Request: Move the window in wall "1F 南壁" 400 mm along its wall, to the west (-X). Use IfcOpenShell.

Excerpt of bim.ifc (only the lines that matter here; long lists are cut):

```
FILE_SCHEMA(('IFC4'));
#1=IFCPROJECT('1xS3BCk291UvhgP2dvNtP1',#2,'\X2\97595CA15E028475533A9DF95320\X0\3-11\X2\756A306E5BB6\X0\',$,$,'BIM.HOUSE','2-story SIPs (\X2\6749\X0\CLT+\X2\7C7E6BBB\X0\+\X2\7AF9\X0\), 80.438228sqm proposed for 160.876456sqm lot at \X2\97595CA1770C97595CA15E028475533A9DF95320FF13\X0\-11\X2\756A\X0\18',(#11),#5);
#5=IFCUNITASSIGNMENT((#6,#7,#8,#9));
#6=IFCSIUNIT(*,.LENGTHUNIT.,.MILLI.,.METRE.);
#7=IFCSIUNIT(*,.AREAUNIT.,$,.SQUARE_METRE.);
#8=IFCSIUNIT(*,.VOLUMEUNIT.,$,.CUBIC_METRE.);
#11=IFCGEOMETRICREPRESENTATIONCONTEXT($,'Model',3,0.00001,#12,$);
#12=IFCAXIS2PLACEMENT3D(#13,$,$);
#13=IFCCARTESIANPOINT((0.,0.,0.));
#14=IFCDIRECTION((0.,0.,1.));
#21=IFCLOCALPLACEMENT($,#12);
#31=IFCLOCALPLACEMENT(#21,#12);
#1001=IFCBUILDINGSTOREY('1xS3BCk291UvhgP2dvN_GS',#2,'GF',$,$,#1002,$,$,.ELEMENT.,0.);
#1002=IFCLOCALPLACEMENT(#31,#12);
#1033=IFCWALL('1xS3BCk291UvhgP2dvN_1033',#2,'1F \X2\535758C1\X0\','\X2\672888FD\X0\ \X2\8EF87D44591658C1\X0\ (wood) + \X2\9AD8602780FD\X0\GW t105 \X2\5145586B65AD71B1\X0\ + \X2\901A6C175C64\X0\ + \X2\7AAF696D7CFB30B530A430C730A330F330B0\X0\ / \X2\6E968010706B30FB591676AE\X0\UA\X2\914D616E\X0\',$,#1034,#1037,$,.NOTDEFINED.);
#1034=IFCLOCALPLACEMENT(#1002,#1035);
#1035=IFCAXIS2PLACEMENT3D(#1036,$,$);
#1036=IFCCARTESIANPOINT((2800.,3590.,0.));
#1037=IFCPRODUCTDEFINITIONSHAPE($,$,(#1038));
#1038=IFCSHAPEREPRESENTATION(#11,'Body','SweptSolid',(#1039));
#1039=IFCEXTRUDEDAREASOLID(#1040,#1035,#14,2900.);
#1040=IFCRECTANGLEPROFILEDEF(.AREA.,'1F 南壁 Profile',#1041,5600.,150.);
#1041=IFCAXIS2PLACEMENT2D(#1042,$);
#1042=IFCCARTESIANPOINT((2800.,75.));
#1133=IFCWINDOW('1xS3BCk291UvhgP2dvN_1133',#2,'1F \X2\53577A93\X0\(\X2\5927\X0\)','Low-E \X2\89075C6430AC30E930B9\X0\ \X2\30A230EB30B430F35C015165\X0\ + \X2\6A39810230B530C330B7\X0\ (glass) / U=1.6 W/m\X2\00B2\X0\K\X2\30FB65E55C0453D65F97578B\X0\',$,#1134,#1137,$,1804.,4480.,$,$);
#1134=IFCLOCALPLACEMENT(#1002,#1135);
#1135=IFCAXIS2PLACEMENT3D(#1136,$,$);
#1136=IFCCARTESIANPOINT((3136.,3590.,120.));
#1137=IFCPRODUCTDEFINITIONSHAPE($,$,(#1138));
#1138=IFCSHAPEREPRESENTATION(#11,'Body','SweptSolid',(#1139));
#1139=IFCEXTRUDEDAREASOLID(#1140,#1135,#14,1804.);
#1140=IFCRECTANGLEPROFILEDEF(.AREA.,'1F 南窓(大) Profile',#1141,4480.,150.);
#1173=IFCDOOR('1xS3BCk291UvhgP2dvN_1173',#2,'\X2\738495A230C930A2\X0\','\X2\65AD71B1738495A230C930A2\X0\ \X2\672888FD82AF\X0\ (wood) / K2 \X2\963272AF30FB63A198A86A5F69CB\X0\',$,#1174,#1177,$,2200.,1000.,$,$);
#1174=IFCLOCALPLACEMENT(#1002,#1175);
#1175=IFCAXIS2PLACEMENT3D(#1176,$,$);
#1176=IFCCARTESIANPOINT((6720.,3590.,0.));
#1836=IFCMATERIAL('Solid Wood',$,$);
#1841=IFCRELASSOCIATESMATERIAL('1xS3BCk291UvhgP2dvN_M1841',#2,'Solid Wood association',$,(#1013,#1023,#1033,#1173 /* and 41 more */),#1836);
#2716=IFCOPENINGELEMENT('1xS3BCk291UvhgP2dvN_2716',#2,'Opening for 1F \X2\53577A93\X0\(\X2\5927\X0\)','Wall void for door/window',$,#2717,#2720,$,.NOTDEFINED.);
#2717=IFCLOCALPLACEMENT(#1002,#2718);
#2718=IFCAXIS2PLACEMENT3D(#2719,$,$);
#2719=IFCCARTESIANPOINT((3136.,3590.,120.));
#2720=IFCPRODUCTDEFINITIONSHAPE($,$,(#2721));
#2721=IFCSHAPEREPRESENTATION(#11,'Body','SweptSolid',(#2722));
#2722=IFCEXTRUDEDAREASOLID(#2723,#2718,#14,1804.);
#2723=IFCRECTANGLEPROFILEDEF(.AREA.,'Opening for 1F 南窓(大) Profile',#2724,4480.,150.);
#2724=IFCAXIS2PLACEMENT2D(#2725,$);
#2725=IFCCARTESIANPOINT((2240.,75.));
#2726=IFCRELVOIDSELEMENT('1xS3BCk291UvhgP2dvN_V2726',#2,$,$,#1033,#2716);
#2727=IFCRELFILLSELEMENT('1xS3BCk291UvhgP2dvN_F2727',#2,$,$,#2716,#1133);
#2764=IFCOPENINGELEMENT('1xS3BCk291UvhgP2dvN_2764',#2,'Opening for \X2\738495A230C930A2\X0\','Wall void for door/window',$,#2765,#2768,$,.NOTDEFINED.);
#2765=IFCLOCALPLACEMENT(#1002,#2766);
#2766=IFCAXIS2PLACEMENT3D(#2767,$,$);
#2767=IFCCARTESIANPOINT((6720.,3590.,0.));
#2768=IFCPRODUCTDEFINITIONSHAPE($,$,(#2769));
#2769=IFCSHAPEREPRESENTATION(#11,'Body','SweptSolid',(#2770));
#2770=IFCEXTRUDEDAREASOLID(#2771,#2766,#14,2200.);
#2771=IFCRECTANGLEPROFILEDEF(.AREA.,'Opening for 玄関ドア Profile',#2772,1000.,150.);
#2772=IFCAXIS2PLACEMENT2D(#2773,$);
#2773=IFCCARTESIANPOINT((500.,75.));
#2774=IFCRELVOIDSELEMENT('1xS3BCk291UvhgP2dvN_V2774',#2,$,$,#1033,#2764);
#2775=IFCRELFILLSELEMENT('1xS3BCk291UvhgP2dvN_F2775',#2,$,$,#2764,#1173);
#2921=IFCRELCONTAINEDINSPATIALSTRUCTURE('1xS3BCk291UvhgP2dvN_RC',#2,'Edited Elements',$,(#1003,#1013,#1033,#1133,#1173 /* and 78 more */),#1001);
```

```python
import ifcopenshell
import ifcopenshell.api.geometry
import ifcopenshell.util.placement
import ifcopenshell.util.unit

model = ifcopenshell.open("bim.ifc")
unit_scale = ifcopenshell.util.unit.calculate_unit_scale(model)

window = model.by_guid("1xS3BCk291UvhgP2dvN_1133")
opening = window.FillsVoids[0].RelatingOpeningElement
wall = opening.VoidsElements[0].RelatingBuildingElement

wall_matrix = ifcopenshell.util.placement.get_local_placement(wall.ObjectPlacement)
shift = wall_matrix[:3, 0] * -0.4 / unit_scale
before = ifcopenshell.util.placement.get_local_placement(window.ObjectPlacement)[:3, 3].copy()

# The window is not placed relative to its opening, so move both.
for product in (opening, window):
    matrix = ifcopenshell.util.placement.get_local_placement(product.ObjectPlacement)
    matrix[:3, 3] += shift
    ifcopenshell.api.geometry.edit_object_placement(model, product=product, matrix=matrix, is_si=False)

after = ifcopenshell.util.placement.get_local_placement(window.ObjectPlacement)[:3, 3]
print("window moved by", (after - before).round(3) + 0.0)

model.write("bim-out.ifc")
```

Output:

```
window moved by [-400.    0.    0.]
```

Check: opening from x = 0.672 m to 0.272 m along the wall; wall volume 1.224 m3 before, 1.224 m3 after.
